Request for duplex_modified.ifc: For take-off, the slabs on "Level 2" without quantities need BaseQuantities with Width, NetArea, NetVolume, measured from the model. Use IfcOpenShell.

First a look at what the model holds.

```python
import ifcopenshell
import ifcopenshell.util.element
import ifcopenshell.util.unit

model = ifcopenshell.open("duplex_modified.ifc")
print(model.schema)
for unit_type in ("LENGTHUNIT", "AREAUNIT", "VOLUMEUNIT"):
    print(unit_type, ifcopenshell.util.unit.calculate_unit_scale(model, unit_type))
storey = next(s for s in model.by_type("IfcBuildingStorey") if s.Name == "Level 2")
slabs = [e for e in ifcopenshell.util.element.get_decomposition(storey) if e.is_a("IfcSlab")]
for e in sorted(slabs, key=lambda e: e.id()):
    print(e.id(), e.is_a(), e.Name, list(ifcopenshell.util.element.get_psets(e, qtos_only=True)), sep=" | ")
```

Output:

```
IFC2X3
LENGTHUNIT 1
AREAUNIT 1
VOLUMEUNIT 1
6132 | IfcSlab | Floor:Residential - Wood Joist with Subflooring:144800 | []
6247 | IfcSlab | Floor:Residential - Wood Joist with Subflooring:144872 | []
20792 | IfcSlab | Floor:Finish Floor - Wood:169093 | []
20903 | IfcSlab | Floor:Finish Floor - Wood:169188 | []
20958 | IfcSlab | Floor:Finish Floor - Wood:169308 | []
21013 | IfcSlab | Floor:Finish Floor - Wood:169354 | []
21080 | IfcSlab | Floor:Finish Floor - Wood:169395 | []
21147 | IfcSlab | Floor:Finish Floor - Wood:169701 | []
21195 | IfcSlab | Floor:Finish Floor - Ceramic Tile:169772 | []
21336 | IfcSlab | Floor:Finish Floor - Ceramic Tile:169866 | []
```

```python
import ifcopenshell
import ifcopenshell.api.pset
import ifcopenshell.geom
import ifcopenshell.util.element
import ifcopenshell.util.shape
import ifcopenshell.util.unit

model = ifcopenshell.open("duplex_modified.ifc")
unit_scale = ifcopenshell.util.unit.calculate_unit_scale(model)
area_scale = ifcopenshell.util.unit.calculate_unit_scale(model, "AREAUNIT")
volume_scale = ifcopenshell.util.unit.calculate_unit_scale(model, "VOLUMEUNIT")
settings = ifcopenshell.geom.settings()

storey = next(s for s in model.by_type("IfcBuildingStorey") if s.Name == "Level 2")
slabs = [e for e in ifcopenshell.util.element.get_decomposition(storey) if e.is_a("IfcSlab")]

for e in sorted(slabs, key=lambda e: e.id()):
    if ifcopenshell.util.element.get_psets(e, qtos_only=True, should_inherit=False):
        continue
    # Geometry comes back in metres, in the element's own axes.
    shape = ifcopenshell.geom.create_shape(settings, e)
    values = {
        "Width": ifcopenshell.util.shape.get_z(shape.geometry) / unit_scale,
        "NetArea": ifcopenshell.util.shape.get_footprint_area(shape.geometry) / area_scale,
        "NetVolume": ifcopenshell.util.shape.get_volume(shape.geometry) / volume_scale,
    }
    qto = ifcopenshell.api.pset.add_qto(model, product=e, name="BaseQuantities")
    ifcopenshell.api.pset.edit_qto(model, qto=qto, properties=values)
    print(e.id(), {k: round(v, 3) for k, v in values.items()})

model.write("duplex_modified_rev.ifc")
```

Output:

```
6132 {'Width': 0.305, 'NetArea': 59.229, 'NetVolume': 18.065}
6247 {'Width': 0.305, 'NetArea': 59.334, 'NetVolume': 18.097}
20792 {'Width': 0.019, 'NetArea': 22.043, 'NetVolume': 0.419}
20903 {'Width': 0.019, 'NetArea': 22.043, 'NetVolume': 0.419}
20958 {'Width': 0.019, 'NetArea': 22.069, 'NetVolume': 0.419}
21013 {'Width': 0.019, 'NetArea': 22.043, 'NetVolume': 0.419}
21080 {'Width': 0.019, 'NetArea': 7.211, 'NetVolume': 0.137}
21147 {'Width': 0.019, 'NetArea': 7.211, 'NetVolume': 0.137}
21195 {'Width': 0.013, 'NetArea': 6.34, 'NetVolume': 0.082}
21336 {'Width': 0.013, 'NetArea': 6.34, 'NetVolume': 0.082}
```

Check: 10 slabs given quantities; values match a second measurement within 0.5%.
